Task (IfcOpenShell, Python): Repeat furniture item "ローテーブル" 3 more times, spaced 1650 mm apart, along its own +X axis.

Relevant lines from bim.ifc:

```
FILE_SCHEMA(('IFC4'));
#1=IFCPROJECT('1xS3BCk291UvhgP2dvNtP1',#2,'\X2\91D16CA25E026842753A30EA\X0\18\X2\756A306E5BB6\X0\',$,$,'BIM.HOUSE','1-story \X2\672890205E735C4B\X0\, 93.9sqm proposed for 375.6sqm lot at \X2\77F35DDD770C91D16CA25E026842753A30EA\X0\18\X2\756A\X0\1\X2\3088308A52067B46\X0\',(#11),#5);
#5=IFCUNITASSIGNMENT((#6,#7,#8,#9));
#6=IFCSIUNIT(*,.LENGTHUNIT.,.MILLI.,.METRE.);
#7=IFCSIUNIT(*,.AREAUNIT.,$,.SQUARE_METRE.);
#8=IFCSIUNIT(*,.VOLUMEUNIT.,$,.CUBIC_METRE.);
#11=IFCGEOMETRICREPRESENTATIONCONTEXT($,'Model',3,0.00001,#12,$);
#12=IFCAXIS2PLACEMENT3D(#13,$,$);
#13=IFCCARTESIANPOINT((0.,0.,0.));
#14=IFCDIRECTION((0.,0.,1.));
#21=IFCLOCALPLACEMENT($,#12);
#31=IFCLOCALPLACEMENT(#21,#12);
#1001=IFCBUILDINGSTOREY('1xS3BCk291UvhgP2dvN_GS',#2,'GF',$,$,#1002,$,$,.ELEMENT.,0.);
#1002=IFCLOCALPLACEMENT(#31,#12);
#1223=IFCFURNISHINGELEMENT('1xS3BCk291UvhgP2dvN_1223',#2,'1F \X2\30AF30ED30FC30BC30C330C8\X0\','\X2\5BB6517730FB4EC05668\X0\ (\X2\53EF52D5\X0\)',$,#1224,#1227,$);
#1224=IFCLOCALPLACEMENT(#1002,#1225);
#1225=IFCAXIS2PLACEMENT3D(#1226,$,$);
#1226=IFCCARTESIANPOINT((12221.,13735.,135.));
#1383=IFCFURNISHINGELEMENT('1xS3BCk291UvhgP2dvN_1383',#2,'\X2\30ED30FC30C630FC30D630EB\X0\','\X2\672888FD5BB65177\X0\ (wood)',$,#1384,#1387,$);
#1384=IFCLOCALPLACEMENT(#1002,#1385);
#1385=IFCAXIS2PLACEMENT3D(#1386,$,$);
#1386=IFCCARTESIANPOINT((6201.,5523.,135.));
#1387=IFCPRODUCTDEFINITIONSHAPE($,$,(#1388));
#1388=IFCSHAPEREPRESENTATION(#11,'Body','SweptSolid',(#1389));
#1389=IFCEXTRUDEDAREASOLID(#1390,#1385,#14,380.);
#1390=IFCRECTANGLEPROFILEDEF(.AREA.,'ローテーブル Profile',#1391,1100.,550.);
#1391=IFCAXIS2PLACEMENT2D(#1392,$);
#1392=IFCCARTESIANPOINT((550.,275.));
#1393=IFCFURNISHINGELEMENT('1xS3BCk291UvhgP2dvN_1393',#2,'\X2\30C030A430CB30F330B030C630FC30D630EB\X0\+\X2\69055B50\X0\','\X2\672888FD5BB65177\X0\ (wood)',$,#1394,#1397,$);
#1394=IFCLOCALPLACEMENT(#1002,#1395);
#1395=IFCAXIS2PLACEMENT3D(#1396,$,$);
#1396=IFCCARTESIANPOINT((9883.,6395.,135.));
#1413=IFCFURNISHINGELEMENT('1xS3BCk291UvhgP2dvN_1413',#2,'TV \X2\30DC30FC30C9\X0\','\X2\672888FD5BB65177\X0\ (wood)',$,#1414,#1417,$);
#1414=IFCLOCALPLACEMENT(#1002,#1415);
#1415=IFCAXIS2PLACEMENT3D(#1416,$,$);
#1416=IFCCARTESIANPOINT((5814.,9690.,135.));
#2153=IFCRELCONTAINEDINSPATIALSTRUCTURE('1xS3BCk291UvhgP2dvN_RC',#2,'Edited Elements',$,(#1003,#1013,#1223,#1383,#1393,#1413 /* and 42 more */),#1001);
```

```python
import ifcopenshell
import ifcopenshell.api.geometry
import ifcopenshell.api.root
import ifcopenshell.util.element
import ifcopenshell.util.placement

model = ifcopenshell.open("bim.ifc")


def reuse_history(source, copy):
    """copy_class also copies each property set's owner history, people and application; keep the originals."""
    for rel in copy.IsDefinedBy:
        if rel.is_a("IfcRelDefinesByProperties") and (history := rel.RelatingPropertyDefinition.OwnerHistory):
            rel.RelatingPropertyDefinition.OwnerHistory = source.OwnerHistory
            ifcopenshell.util.element.remove_deep2(model, history)


source = model.by_id(1383)
base = ifcopenshell.util.placement.get_local_placement(source.ObjectPlacement)
step = base[:3, 0] * 1650.0

for i in range(1, 4):
    copy = ifcopenshell.api.root.copy_class(model, product=source)
    copy.Representation = ifcopenshell.util.element.copy_deep(
        model, source.Representation, exclude=["IfcGeometricRepresentationContext", "IfcRepresentationMap"]
    )
    reuse_history(source, copy)
    matrix = base.copy()
    matrix[:3, 3] += i * step
    print("added at", matrix[:3, 3].round(3) + 0.0)
    ifcopenshell.api.geometry.edit_object_placement(model, product=copy, matrix=matrix, is_si=False)

model.write("bim_rev.ifc")
```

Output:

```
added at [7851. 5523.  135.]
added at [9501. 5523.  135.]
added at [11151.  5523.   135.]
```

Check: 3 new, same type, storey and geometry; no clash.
